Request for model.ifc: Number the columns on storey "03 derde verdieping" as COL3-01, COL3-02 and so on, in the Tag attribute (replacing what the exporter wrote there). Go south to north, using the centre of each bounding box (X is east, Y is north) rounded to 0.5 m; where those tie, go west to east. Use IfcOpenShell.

First a look at what the model holds.

```python
import ifcopenshell
import ifcopenshell.util.element
import ifcopenshell.util.placement

model = ifcopenshell.open("model.ifc")
print(model.schema)
storey = next(s for s in model.by_type("IfcBuildingStorey") if s.Name == "03 derde verdieping")
columns = [e for e in ifcopenshell.util.element.get_decomposition(storey) if e.is_a("IfcColumn")]
for e in sorted(columns, key=lambda e: e.id()):
    origin = ifcopenshell.util.placement.get_local_placement(e.ObjectPlacement)[:3, 3]
    print(e.id(), e.Tag, e.Name, origin.round(2) + 0.0, sep=" | ")
```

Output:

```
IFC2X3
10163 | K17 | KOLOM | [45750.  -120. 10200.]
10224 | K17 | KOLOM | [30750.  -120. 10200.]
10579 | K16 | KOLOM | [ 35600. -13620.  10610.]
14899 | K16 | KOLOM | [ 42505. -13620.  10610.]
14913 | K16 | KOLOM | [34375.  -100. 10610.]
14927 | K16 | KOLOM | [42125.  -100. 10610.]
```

```python
import ifcopenshell
import ifcopenshell.geom
import ifcopenshell.util.element
import ifcopenshell.util.shape

model = ifcopenshell.open("model.ifc")
settings = ifcopenshell.geom.settings()
settings.set("use-world-coords", True)


def centre(element):
    shape = ifcopenshell.geom.create_shape(settings, element)
    return ifcopenshell.util.shape.get_bbox_centroid(shape.geometry)


storey = next(s for s in model.by_type("IfcBuildingStorey") if s.Name == "03 derde verdieping")
columns = [e for e in ifcopenshell.util.element.get_decomposition(storey) if e.is_a("IfcColumn")]

# Insertion points can sit at a corner or the storey origin, so sort by the geometry (in metres).
centres = {e: centre(e) for e in columns}
columns.sort(key=lambda e: (round(centres[e][1] / 0.5), centres[e][0]))

for i, e in enumerate(columns, start=1):
    number = f"COL3-{i:02d}"
    e.Tag = number
    print(e.id(), number)

model.write("model_v2.ifc")
```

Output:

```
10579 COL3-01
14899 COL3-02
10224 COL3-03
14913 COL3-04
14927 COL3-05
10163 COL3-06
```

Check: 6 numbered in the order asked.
